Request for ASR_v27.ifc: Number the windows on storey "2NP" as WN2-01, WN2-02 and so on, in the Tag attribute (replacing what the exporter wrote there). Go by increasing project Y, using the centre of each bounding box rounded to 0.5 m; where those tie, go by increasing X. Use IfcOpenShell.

First a look at what the model holds.

```python
import ifcopenshell
import ifcopenshell.util.element
import ifcopenshell.util.placement

model = ifcopenshell.open("ASR_v27.ifc")
print(model.schema)
storey = next(s for s in model.by_type("IfcBuildingStorey") if s.Name == "2NP")
windows = [e for e in ifcopenshell.util.element.get_decomposition(storey) if e.is_a("IfcWindow")]
for e in sorted(windows, key=lambda e: e.id()):
    origin = ifcopenshell.util.placement.get_local_placement(e.ObjectPlacement)[:3, 3]
    print(e.id(), e.Tag, e.Name, origin.round(2) + 0.0, sep=" | ")
```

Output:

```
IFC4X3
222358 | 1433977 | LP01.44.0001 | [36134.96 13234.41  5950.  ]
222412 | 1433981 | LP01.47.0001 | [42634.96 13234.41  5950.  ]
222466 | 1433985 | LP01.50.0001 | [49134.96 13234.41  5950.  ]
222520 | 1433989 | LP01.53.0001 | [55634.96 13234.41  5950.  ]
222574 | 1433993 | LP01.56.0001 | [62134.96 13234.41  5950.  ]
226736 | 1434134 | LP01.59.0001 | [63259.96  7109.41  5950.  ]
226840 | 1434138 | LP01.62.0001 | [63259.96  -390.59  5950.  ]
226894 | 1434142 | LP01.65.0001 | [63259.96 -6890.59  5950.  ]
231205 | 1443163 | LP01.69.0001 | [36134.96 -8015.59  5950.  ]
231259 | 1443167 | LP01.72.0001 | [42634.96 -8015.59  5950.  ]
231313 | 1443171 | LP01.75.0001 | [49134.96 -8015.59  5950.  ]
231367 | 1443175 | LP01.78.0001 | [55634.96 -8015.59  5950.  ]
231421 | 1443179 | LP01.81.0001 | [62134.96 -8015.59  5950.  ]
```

```python
import ifcopenshell
import ifcopenshell.geom
import ifcopenshell.util.element
import ifcopenshell.util.shape

model = ifcopenshell.open("ASR_v27.ifc")
settings = ifcopenshell.geom.settings()
settings.set("use-world-coords", True)


def centre(element):
    shape = ifcopenshell.geom.create_shape(settings, element)
    return ifcopenshell.util.shape.get_bbox_centroid(shape.geometry)


storey = next(s for s in model.by_type("IfcBuildingStorey") if s.Name == "2NP")
windows = [e for e in ifcopenshell.util.element.get_decomposition(storey) if e.is_a("IfcWindow")]

# Insertion points can sit at a corner or the storey origin, so sort by the geometry (in metres).
centres = {e: centre(e) for e in windows}
windows.sort(key=lambda e: (round(centres[e][1] / 0.5), centres[e][0]))

for i, e in enumerate(windows, start=1):
    number = f"WN2-{i:02d}"
    e.Tag = number
    print(e.id(), number)

model.write("ASR_v27_v2.ifc")
```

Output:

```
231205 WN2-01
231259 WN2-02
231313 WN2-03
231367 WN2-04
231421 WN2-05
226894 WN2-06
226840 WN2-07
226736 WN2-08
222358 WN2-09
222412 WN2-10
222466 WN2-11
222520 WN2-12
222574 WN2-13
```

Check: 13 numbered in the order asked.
